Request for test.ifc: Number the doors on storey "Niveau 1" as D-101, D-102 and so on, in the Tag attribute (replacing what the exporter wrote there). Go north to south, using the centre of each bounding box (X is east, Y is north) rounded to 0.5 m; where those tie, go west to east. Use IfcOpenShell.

First a look at what the model holds.

```python
import ifcopenshell
import ifcopenshell.util.element
import ifcopenshell.util.placement

model = ifcopenshell.open("test.ifc")
print(model.schema)
storey = next(s for s in model.by_type("IfcBuildingStorey") if s.Name == "Niveau 1")
doors = [e for e in ifcopenshell.util.element.get_decomposition(storey) if e.is_a("IfcDoor")]
for e in sorted(doors, key=lambda e: e.id()):
    origin = ifcopenshell.util.placement.get_local_placement(e.ObjectPlacement)[:3, 3]
    print(e.id(), e.Tag, e.Name, origin.round(2) + 0.0, sep=" | ")
```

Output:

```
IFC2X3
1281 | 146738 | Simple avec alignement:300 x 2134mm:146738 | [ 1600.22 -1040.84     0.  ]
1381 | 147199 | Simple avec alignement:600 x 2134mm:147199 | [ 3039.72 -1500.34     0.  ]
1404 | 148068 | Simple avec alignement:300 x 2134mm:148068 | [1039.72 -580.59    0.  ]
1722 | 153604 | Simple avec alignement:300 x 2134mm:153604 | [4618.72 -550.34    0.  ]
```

```python
import ifcopenshell
import ifcopenshell.geom
import ifcopenshell.util.element
import ifcopenshell.util.shape

model = ifcopenshell.open("test.ifc")
settings = ifcopenshell.geom.settings()
settings.set("use-world-coords", True)


def centre(element):
    shape = ifcopenshell.geom.create_shape(settings, element)
    return ifcopenshell.util.shape.get_bbox_centroid(shape.geometry)


storey = next(s for s in model.by_type("IfcBuildingStorey") if s.Name == "Niveau 1")
doors = [e for e in ifcopenshell.util.element.get_decomposition(storey) if e.is_a("IfcDoor")]

# Insertion points can sit at a corner or the storey origin, so sort by the geometry (in metres).
centres = {e: centre(e) for e in doors}
doors.sort(key=lambda e: (-round(centres[e][1] / 0.5), centres[e][0]))

for i, e in enumerate(doors, start=1):
    number = f"D-1{i:02d}"
    e.Tag = number
    print(e.id(), number)

model.write("test-out.ifc")
```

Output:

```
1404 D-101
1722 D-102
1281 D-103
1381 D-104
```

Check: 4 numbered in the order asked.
